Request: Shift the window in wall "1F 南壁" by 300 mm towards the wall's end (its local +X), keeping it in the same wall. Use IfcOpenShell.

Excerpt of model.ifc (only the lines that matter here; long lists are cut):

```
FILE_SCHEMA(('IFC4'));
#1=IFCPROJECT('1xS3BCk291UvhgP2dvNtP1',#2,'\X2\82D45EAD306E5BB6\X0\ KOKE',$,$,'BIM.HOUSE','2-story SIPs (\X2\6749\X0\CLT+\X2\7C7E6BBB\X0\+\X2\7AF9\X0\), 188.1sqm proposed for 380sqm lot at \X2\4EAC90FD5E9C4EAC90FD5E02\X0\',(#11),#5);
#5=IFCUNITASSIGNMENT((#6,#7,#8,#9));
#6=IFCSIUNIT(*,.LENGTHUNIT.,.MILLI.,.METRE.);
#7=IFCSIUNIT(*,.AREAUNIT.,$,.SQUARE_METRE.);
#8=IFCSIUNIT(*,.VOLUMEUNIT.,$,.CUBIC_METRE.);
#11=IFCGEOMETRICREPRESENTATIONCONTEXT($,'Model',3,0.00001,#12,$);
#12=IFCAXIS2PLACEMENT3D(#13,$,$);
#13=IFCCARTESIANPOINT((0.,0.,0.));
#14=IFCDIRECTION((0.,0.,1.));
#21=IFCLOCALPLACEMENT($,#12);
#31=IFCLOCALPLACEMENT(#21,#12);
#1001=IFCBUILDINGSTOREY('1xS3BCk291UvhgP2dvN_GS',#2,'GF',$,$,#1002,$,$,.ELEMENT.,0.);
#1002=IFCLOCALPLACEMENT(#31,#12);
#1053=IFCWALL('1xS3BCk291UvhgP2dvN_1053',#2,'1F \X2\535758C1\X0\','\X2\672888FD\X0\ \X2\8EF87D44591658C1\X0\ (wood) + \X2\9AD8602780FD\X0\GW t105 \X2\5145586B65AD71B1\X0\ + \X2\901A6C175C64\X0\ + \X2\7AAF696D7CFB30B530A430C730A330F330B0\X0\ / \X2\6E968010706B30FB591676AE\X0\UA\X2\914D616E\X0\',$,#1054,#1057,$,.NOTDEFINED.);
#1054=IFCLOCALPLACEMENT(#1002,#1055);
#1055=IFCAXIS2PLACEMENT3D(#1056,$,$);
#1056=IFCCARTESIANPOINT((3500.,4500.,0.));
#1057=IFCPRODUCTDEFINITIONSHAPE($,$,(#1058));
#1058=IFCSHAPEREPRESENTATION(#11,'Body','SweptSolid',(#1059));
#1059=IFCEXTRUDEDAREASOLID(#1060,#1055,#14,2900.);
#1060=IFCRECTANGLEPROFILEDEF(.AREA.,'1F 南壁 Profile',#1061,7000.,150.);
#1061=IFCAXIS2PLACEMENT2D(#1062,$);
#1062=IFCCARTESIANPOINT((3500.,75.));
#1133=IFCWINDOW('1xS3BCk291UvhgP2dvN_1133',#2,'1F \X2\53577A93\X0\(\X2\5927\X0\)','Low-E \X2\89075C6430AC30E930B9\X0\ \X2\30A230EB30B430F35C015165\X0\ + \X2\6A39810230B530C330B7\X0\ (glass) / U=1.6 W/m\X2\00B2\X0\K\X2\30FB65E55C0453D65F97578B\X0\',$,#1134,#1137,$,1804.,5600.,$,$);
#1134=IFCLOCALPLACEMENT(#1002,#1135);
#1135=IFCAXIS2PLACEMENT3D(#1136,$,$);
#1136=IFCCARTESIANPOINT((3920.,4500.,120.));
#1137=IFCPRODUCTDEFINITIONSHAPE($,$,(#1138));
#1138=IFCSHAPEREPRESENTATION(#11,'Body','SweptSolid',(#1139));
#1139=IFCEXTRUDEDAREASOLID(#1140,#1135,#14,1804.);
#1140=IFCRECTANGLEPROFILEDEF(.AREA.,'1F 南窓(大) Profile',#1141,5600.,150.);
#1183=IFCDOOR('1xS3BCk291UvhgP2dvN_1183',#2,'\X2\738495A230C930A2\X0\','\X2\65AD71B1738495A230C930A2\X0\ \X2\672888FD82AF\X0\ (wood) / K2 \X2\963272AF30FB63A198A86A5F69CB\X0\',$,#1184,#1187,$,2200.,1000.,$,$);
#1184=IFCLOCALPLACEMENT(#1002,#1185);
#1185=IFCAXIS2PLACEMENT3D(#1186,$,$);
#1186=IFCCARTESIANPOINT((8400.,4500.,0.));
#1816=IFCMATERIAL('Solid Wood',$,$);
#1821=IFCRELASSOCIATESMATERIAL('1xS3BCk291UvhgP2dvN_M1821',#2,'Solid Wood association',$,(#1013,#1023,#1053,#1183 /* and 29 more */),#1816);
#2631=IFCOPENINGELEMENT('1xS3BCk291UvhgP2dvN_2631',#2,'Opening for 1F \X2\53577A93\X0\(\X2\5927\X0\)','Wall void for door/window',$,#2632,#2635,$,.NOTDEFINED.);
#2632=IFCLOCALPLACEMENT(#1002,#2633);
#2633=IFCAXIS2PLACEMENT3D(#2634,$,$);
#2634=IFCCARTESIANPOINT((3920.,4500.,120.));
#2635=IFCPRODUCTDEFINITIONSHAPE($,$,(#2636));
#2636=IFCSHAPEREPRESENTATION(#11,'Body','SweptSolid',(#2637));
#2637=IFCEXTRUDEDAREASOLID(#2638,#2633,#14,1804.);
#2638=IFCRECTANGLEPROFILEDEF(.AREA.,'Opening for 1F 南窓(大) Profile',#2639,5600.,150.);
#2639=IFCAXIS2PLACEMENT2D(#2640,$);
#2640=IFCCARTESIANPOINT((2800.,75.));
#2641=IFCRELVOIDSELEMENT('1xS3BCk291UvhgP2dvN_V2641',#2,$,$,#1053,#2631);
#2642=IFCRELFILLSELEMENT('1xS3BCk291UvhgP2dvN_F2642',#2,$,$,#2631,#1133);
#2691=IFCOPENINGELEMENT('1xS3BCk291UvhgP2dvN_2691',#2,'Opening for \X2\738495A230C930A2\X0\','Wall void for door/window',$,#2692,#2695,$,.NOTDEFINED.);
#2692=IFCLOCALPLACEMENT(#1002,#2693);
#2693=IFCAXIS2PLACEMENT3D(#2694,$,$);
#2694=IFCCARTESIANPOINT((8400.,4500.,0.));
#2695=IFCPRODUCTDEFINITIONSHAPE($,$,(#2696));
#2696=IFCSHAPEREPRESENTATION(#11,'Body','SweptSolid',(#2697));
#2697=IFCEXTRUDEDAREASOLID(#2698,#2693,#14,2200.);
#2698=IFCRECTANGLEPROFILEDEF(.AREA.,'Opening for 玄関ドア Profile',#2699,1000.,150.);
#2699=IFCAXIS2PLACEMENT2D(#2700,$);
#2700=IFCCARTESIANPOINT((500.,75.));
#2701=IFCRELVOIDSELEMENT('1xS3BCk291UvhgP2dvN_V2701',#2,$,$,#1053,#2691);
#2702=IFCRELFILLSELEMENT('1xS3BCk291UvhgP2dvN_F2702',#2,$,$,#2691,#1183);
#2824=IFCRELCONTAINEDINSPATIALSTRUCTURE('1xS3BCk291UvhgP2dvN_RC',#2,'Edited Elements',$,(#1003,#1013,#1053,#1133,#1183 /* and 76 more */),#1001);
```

```python
import ifcopenshell
import ifcopenshell.api.geometry
import ifcopenshell.util.placement
import ifcopenshell.util.unit

model = ifcopenshell.open("model.ifc")
unit_scale = ifcopenshell.util.unit.calculate_unit_scale(model)

window = model.by_guid("1xS3BCk291UvhgP2dvN_1133")
opening = window.FillsVoids[0].RelatingOpeningElement
wall = opening.VoidsElements[0].RelatingBuildingElement

wall_matrix = ifcopenshell.util.placement.get_local_placement(wall.ObjectPlacement)
shift = wall_matrix[:3, 0] * 0.3 / unit_scale
before = ifcopenshell.util.placement.get_local_placement(window.ObjectPlacement)[:3, 3].copy()

# The window is not placed relative to its opening, so move both.
for product in (opening, window):
    matrix = ifcopenshell.util.placement.get_local_placement(product.ObjectPlacement)
    matrix[:3, 3] += shift
    ifcopenshell.api.geometry.edit_object_placement(model, product=product, matrix=matrix, is_si=False)

after = ifcopenshell.util.placement.get_local_placement(window.ObjectPlacement)[:3, 3]
print("window moved by", (after - before).round(3) + 0.0)

model.write("model_rev.ifc")
```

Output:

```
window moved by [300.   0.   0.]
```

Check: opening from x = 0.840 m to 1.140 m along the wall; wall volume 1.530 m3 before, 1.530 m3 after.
